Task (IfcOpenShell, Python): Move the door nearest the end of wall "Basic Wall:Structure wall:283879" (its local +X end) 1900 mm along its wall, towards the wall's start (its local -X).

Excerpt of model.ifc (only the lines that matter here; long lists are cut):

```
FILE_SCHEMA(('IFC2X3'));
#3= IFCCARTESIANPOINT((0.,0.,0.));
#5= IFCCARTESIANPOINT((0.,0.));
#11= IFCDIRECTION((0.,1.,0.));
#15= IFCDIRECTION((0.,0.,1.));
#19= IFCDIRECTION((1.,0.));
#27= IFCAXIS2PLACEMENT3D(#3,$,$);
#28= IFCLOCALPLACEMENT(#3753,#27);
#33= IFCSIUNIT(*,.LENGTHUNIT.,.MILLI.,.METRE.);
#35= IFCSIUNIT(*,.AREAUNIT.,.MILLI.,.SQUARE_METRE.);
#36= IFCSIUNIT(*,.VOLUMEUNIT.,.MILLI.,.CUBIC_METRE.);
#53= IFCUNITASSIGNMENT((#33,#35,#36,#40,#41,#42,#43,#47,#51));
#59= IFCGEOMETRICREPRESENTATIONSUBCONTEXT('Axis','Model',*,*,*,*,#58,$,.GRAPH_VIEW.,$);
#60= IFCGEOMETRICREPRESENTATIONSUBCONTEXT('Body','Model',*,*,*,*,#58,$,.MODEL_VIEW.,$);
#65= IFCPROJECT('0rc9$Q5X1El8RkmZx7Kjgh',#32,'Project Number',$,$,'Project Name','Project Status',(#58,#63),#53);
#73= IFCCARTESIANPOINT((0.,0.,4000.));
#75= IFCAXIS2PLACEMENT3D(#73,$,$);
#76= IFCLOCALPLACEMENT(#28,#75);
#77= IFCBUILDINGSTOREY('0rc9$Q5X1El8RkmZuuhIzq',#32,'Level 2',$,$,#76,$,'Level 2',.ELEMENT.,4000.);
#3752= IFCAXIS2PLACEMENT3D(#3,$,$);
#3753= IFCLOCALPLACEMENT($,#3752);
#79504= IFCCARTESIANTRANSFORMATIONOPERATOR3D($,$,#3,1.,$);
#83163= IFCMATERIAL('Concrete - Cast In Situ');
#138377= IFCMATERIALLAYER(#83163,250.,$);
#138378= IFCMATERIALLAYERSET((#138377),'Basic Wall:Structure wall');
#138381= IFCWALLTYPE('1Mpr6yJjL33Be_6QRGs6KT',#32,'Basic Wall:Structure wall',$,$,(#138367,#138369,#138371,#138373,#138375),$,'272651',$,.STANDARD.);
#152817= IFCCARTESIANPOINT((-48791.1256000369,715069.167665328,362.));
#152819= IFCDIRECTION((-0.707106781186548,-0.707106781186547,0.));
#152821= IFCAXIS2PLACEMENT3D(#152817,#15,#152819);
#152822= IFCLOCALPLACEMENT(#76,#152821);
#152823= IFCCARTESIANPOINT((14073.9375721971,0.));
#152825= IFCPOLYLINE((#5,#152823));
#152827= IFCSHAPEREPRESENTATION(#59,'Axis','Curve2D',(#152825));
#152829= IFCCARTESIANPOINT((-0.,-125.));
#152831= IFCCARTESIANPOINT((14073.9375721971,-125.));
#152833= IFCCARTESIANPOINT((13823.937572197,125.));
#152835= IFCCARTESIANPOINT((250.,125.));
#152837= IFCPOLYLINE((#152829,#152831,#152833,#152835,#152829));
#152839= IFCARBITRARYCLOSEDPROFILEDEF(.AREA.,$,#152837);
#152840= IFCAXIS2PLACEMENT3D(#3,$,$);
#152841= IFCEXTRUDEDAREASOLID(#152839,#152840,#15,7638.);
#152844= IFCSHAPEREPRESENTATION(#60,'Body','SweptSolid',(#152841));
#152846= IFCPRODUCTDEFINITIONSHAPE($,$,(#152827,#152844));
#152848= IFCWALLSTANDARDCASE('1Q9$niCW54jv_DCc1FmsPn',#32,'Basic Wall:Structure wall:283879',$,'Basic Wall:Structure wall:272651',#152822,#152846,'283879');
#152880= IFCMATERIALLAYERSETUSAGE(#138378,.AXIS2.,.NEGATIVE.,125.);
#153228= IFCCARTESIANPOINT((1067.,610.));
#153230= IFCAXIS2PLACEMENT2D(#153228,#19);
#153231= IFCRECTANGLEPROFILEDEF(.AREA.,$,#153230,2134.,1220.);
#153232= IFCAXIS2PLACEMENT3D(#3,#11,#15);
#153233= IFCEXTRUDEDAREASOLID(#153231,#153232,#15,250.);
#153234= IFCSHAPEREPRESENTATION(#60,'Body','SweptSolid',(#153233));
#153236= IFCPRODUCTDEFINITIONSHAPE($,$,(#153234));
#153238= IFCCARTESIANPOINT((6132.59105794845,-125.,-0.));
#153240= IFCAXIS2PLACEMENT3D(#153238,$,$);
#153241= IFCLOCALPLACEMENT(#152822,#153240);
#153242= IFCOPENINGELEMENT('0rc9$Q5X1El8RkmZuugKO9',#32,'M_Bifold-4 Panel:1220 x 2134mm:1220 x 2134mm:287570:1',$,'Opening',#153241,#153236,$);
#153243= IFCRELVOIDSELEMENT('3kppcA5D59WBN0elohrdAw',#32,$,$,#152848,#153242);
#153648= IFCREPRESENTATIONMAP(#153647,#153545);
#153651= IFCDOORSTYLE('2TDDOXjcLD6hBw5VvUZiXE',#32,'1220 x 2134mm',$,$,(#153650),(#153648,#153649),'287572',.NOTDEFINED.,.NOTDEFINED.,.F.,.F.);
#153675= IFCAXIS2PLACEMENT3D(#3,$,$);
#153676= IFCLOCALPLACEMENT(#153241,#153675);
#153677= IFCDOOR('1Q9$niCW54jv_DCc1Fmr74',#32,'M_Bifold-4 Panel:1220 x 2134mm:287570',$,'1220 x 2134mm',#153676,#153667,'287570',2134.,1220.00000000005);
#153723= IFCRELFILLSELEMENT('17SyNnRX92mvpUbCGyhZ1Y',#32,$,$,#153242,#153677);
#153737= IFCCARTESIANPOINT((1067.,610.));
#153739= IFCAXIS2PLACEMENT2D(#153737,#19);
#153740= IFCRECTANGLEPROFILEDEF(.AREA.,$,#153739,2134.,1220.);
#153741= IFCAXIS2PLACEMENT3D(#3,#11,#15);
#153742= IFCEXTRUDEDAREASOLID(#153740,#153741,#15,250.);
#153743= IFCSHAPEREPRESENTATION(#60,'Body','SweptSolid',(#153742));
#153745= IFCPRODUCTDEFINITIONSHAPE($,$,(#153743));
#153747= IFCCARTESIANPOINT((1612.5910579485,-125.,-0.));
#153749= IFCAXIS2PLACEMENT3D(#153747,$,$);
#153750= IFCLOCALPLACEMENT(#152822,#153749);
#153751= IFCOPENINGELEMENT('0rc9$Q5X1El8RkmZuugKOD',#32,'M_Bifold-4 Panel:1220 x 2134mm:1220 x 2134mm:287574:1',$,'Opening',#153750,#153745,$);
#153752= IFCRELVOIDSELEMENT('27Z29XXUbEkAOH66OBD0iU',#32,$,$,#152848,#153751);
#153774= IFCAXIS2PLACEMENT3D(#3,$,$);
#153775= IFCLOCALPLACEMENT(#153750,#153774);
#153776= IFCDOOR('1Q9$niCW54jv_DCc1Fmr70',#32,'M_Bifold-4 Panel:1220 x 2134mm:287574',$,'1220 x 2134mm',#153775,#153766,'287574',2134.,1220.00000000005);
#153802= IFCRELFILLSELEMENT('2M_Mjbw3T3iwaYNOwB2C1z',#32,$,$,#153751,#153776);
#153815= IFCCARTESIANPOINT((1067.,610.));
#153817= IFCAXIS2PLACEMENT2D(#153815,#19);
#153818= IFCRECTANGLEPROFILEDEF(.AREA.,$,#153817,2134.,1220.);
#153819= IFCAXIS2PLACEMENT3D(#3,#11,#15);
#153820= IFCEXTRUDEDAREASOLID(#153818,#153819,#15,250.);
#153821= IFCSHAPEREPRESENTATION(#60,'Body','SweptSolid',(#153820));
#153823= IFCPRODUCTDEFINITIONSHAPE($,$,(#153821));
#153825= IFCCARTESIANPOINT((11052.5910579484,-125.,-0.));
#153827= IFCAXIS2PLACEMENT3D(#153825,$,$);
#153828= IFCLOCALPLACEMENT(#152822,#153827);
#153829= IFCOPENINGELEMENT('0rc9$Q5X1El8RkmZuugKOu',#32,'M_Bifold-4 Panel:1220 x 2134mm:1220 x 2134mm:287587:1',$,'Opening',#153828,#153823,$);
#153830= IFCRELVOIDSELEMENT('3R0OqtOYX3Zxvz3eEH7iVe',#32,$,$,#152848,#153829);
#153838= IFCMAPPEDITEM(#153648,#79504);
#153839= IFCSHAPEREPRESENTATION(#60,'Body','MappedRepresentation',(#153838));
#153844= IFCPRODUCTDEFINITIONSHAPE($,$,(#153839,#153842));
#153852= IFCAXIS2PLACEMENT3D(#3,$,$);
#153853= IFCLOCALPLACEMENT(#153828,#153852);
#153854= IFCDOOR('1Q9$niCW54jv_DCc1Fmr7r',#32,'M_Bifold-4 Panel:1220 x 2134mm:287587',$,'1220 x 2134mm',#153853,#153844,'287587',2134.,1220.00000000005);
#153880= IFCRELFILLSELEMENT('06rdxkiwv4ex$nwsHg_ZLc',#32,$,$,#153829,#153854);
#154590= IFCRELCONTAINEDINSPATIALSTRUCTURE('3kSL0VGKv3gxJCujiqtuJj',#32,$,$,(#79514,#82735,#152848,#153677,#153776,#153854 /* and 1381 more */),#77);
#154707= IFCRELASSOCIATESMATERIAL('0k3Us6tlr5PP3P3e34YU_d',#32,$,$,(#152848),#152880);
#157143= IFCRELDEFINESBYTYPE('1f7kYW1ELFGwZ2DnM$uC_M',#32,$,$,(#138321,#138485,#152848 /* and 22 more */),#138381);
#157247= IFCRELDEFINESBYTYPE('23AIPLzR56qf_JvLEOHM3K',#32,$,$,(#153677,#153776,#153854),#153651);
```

```python
import ifcopenshell
import ifcopenshell.api.geometry
import ifcopenshell.util.placement
import ifcopenshell.util.unit

model = ifcopenshell.open("model.ifc")
unit_scale = ifcopenshell.util.unit.calculate_unit_scale(model)

door = model.by_guid("1Q9$niCW54jv_DCc1Fmr7r")
opening = door.FillsVoids[0].RelatingOpeningElement
wall = opening.VoidsElements[0].RelatingBuildingElement

wall_matrix = ifcopenshell.util.placement.get_local_placement(wall.ObjectPlacement)
shift = wall_matrix[:3, 0] * -1.9 / unit_scale
before = ifcopenshell.util.placement.get_local_placement(door.ObjectPlacement)[:3, 3].copy()

# The door is placed relative to its opening, so it follows when the opening moves.
matrix = ifcopenshell.util.placement.get_local_placement(opening.ObjectPlacement)
matrix[:3, 3] += shift
ifcopenshell.api.geometry.edit_object_placement(
    model, product=opening, matrix=matrix, is_si=False, should_transform_children=True
)

after = ifcopenshell.util.placement.get_local_placement(door.ObjectPlacement)[:3, 3]
print("door moved by", (after - before).round(3) + 0.0)

model.write("model_rev.ifc")
```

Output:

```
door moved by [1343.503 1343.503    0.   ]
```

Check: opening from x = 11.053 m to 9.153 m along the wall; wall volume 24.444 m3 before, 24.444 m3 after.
